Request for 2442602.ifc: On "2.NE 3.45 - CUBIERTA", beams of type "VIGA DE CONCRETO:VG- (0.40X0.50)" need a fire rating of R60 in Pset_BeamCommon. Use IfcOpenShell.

First a look at what the model holds.

```python
import ifcopenshell
import ifcopenshell.util.element

model = ifcopenshell.open("2442602.ifc")
print(model.schema)
storey = next(s for s in model.by_type("IfcBuildingStorey") if s.Name == "2.NE 3.45 - CUBIERTA")
beams = [e for e in ifcopenshell.util.element.get_decomposition(storey) if e.is_a("IfcBeam")]
seen = {}
for e in beams:
    element_type = ifcopenshell.util.element.get_type(e)
    key = (element_type.Name if element_type != e and element_type else None, ifcopenshell.util.element.get_pset(e, "Pset_BeamCommon", "FireRating"))
    seen[key] = seen.get(key, 0) + 1
for (name, value), count in sorted(seen.items(), key=str):
    print(count, "x", name, "|", value)
```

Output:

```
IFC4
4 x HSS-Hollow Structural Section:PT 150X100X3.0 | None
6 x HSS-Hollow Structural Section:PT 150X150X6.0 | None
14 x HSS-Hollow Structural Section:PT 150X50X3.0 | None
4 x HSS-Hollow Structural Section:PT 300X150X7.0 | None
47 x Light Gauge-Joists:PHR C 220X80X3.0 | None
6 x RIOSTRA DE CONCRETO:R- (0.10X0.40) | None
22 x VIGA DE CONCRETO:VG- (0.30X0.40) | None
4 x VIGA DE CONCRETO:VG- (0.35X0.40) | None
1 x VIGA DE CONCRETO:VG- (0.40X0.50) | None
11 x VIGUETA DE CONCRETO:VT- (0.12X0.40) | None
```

```python
import ifcopenshell
import ifcopenshell.api.pset
import ifcopenshell.util.element

model = ifcopenshell.open("2442602.ifc")

storey = next(s for s in model.by_type("IfcBuildingStorey") if s.Name == "2.NE 3.45 - CUBIERTA")
beams = [e for e in ifcopenshell.util.element.get_decomposition(storey) if e.is_a("IfcBeam")]

count = 0
for e in beams:
    element_type = ifcopenshell.util.element.get_type(e)
    if element_type in (None, e) or element_type.Name != "VIGA DE CONCRETO:VG- (0.40X0.50)":
        continue
    # add_pset returns the element's existing set when there is one.
    pset = ifcopenshell.api.pset.add_pset(model, product=e, name="Pset_BeamCommon")
    ifcopenshell.api.pset.edit_pset(model, pset=pset, properties={"FireRating": "R60"})
    count += 1

print(count, "beams updated")

model.write("2442602_rev.ifc")
```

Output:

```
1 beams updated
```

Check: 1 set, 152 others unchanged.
